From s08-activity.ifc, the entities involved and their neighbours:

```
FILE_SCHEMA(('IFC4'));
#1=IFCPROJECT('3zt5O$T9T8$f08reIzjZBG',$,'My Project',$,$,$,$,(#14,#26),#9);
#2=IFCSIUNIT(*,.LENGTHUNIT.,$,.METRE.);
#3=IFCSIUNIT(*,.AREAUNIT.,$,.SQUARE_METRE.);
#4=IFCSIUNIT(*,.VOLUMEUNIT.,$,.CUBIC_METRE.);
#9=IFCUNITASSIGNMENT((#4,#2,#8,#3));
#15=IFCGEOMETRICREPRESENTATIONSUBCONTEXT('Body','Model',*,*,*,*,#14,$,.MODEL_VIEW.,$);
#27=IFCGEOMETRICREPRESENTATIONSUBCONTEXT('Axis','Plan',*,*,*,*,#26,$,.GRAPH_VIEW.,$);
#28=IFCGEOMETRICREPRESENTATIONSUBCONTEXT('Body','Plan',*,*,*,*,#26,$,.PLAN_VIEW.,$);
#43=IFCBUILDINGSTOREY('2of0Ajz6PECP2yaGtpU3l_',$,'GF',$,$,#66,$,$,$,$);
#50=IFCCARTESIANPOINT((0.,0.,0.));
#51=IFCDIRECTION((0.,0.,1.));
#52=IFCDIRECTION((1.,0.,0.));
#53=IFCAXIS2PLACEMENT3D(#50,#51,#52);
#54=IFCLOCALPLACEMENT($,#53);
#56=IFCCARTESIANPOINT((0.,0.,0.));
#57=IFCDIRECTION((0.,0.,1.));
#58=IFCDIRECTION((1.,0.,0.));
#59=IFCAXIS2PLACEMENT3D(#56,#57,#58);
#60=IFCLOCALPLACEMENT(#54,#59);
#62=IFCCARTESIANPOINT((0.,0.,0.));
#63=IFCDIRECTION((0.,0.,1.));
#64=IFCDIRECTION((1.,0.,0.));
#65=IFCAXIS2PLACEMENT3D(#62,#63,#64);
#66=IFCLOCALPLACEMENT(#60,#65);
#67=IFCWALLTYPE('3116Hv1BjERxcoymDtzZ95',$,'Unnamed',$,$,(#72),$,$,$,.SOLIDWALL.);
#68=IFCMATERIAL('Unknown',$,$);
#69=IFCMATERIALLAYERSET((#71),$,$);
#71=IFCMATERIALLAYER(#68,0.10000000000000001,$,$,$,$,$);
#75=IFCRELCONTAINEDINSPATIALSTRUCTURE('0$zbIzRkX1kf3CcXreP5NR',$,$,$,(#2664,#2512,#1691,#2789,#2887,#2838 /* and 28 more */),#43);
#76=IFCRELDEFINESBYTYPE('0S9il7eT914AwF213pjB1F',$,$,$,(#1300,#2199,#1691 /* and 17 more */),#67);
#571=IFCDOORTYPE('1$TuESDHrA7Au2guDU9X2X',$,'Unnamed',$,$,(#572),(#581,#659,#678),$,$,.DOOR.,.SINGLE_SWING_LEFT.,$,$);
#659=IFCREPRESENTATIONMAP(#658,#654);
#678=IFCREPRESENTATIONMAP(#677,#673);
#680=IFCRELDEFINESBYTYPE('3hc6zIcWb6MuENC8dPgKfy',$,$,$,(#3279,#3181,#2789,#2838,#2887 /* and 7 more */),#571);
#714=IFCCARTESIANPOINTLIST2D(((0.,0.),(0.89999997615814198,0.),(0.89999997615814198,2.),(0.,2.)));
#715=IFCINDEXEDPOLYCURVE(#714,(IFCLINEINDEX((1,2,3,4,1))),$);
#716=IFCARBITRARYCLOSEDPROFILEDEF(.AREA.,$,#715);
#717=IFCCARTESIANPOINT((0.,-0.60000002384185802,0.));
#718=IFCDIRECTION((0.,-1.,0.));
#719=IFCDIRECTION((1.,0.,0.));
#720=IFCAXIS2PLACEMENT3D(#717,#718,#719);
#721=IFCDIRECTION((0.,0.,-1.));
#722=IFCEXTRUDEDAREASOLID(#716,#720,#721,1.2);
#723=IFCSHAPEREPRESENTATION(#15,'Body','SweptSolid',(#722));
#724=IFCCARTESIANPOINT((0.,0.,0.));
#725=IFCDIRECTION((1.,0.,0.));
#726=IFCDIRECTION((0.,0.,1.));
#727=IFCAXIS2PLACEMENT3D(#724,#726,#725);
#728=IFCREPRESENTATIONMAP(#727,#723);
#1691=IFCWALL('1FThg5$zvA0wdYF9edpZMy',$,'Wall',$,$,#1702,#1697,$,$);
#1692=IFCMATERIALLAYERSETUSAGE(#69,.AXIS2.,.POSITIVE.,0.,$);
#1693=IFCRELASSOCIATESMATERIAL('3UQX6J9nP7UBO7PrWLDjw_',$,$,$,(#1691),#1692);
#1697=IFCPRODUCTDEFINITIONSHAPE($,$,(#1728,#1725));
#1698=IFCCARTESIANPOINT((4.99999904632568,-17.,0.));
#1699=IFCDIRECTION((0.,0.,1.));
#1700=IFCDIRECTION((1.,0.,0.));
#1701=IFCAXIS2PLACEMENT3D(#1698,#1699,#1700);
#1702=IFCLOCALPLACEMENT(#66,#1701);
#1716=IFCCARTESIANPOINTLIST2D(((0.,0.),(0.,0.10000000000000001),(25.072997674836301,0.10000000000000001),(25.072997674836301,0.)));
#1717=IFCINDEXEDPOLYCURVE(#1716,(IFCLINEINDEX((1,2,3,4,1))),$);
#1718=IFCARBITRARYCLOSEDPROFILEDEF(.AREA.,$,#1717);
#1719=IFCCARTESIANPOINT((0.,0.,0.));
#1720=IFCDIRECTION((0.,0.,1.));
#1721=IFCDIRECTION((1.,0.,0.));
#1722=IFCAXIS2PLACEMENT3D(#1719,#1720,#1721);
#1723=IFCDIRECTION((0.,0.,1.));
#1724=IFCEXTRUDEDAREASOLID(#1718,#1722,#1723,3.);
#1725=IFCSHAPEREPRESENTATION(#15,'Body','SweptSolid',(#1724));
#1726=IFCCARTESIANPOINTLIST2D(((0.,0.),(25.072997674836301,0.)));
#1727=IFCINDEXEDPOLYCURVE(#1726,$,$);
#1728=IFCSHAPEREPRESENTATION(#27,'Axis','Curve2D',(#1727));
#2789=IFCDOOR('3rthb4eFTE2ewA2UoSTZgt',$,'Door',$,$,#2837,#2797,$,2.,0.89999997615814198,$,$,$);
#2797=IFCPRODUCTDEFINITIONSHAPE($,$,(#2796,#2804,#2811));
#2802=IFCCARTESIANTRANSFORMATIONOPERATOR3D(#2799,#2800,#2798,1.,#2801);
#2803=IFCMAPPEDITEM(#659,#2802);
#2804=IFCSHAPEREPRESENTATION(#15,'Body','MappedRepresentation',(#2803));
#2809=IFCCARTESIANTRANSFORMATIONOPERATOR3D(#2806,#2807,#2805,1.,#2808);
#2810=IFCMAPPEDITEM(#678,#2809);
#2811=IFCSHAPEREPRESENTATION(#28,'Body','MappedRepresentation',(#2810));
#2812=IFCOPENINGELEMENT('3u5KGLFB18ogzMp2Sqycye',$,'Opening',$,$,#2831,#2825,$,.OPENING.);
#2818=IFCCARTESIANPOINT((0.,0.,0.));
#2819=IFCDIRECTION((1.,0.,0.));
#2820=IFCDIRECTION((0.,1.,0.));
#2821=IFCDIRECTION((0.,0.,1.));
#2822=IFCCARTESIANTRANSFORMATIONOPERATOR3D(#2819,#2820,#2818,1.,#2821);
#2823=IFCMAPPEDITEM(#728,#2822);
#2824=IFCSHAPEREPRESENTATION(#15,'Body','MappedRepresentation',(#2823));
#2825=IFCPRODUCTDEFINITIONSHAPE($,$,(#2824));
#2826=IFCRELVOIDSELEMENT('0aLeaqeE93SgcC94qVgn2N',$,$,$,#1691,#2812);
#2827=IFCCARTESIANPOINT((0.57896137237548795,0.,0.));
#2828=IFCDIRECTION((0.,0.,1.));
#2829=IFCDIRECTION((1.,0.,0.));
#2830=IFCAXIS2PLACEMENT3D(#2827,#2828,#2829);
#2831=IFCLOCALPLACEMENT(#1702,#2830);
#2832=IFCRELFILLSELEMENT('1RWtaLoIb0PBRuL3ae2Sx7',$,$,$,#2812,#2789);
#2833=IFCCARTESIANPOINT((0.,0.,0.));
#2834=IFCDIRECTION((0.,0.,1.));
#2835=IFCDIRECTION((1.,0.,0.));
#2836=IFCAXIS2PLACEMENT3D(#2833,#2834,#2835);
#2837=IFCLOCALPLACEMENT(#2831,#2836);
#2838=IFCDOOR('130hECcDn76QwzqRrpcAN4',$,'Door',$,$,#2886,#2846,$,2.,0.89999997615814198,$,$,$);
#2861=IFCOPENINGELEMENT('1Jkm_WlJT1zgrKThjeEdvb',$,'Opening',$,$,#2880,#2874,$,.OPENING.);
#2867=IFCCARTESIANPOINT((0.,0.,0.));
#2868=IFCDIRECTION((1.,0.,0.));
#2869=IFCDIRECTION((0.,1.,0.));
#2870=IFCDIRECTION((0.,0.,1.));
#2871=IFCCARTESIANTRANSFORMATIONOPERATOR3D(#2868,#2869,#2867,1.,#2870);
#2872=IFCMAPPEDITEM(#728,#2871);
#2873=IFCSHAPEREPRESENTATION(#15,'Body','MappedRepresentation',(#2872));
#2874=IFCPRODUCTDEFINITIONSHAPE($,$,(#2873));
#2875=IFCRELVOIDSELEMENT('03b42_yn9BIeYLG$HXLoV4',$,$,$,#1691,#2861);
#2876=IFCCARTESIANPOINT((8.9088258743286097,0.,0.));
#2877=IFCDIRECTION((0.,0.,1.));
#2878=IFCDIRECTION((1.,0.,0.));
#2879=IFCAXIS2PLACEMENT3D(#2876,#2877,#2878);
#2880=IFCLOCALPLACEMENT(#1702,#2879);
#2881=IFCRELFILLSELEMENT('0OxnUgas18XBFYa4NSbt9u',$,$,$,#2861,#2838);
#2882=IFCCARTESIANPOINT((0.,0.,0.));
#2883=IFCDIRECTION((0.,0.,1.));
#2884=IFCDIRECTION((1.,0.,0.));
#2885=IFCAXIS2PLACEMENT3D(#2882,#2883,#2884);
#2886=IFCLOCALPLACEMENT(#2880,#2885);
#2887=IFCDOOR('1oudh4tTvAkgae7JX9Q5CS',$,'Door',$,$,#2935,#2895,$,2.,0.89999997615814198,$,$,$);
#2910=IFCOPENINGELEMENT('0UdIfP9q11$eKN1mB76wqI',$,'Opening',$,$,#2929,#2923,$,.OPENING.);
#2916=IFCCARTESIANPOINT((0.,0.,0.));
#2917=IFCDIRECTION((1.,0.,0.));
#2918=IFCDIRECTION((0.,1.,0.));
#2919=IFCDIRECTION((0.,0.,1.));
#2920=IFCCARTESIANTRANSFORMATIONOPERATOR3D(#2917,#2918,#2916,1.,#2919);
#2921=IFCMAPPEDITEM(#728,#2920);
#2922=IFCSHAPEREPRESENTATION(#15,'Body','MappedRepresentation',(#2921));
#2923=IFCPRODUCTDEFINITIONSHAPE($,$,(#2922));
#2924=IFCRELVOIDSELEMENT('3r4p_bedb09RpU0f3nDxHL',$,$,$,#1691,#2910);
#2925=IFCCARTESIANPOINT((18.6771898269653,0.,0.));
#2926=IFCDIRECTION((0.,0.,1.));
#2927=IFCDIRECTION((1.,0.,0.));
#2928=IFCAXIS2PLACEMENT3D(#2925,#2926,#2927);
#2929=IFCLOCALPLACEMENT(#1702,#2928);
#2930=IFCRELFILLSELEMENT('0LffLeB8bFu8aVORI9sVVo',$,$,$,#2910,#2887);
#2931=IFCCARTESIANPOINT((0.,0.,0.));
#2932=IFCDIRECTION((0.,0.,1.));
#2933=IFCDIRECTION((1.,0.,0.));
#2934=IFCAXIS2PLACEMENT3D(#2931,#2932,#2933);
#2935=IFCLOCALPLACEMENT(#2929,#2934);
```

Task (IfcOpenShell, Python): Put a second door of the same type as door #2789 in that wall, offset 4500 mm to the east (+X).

```python
import ifcopenshell
import ifcopenshell.api.feature
import ifcopenshell.api.geometry
import ifcopenshell.api.root
import ifcopenshell.geom
import ifcopenshell.util.element
import ifcopenshell.util.placement
import ifcopenshell.util.shape
import ifcopenshell.util.unit

model = ifcopenshell.open("s08-activity.ifc")
unit_scale = ifcopenshell.util.unit.calculate_unit_scale(model)
settings = ifcopenshell.geom.settings()


def volume(element):
    """Net volume in cubic metres, openings subtracted."""
    shape = ifcopenshell.geom.create_shape(settings, element)
    return ifcopenshell.util.shape.get_volume(shape.geometry)


door = model.by_guid("3rthb4eFTE2ewA2UoSTZgt")
opening = door.FillsVoids[0].RelatingOpeningElement
wall = opening.VoidsElements[0].RelatingBuildingElement
before = volume(wall)
shift = ifcopenshell.util.placement.get_local_placement(wall.ObjectPlacement)[:3, 0] * 4.5 / unit_scale

# copy_class copies the void relationship, type, container and properties, but no geometry.
new_opening = ifcopenshell.api.root.copy_class(model, product=opening)
new_opening.Representation = ifcopenshell.util.element.copy_deep(
    model, opening.Representation, exclude=["IfcGeometricRepresentationContext", "IfcRepresentationMap"]
)
new_door = ifcopenshell.api.root.copy_class(model, product=door)
new_door.Representation = ifcopenshell.util.element.copy_deep(
    model, door.Representation, exclude=["IfcGeometricRepresentationContext", "IfcRepresentationMap"]
)
ifcopenshell.api.feature.add_filling(model, opening=new_opening, element=new_door)

for old, new in ((opening, new_opening), (door, new_door)):
    matrix = ifcopenshell.util.placement.get_local_placement(old.ObjectPlacement)
    matrix[:3, 3] += shift
    ifcopenshell.api.geometry.edit_object_placement(model, product=new, matrix=matrix, is_si=False)

after = volume(wall)

print(f"wall volume {before:.3f} -> {after:.3f} m3")

model.write("s08-activity_v2.ifc")
```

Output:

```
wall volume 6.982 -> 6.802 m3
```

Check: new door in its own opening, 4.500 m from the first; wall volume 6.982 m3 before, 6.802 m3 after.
